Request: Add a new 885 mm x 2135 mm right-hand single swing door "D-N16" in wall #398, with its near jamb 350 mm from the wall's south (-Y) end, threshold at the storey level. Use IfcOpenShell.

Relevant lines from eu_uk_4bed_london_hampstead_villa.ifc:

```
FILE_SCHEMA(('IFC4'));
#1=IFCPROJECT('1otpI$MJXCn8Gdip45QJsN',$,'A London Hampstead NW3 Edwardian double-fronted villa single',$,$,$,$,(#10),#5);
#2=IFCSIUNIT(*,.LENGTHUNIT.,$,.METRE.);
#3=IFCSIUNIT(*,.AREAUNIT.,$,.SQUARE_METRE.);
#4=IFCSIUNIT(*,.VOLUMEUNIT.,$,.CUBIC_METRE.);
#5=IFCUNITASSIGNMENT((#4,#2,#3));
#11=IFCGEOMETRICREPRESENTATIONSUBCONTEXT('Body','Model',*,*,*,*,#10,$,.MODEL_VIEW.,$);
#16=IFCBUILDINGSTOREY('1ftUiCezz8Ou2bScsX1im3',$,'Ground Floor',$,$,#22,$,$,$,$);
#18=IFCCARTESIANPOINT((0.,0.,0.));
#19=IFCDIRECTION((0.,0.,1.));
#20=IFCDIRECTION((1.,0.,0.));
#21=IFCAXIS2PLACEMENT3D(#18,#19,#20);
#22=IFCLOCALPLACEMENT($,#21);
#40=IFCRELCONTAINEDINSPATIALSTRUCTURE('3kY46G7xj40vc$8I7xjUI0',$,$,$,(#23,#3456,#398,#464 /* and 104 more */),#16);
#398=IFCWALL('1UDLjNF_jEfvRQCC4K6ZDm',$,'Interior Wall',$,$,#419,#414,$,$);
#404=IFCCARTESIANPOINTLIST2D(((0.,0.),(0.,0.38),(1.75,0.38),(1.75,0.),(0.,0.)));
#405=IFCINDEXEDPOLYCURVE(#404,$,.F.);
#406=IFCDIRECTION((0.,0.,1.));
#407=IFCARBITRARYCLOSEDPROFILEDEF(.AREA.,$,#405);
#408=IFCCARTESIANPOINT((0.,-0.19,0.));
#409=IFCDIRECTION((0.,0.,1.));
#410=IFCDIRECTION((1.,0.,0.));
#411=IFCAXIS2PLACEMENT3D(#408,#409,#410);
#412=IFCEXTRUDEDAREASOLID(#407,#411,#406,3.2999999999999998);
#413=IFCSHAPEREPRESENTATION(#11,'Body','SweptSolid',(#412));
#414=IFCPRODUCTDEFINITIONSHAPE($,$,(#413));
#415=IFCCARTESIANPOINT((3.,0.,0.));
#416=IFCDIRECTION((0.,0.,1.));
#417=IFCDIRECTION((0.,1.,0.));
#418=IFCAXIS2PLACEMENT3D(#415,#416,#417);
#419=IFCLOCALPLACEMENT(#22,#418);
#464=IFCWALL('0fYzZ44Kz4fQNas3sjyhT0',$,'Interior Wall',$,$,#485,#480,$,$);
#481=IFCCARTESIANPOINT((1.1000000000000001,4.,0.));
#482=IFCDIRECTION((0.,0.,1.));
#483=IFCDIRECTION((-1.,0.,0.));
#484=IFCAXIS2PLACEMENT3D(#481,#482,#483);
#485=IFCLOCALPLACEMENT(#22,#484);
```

```python
import numpy as np
import ifcopenshell
import ifcopenshell.api.feature
import ifcopenshell.api.geometry
import ifcopenshell.api.root
import ifcopenshell.api.spatial
import ifcopenshell.geom
import ifcopenshell.util.element
import ifcopenshell.util.placement
import ifcopenshell.util.representation
import ifcopenshell.util.shape
import ifcopenshell.util.unit

model = ifcopenshell.open("eu_uk_4bed_london_hampstead_villa.ifc")
unit_scale = ifcopenshell.util.unit.calculate_unit_scale(model)
settings = ifcopenshell.geom.settings()


def volume(element):
    """Net volume in cubic metres, openings subtracted."""
    shape = ifcopenshell.geom.create_shape(settings, element)
    return ifcopenshell.util.shape.get_volume(shape.geometry)


wall = model.by_guid("1UDLjNF_jEfvRQCC4K6ZDm")
storey = ifcopenshell.util.element.get_container(wall, ifc_class="IfcBuildingStorey")
context = ifcopenshell.util.representation.get_context(model, "Model", "Body", "MODEL_VIEW")
before = volume(wall)

width, height, from_end, sill = 0.885, 2.135, 0.35, 0.0  # metres

# The wall runs along its own X axis, and the end named is its -X end.
wall_shape = ifcopenshell.geom.create_shape(settings, wall)
x, y, z = ifcopenshell.util.shape.get_vertices(wall_shape.geometry).T
start = x.min() + from_end
face, thickness = float(y.min()), float(y.max() - y.min())
wall_matrix = ifcopenshell.util.placement.get_local_placement(wall.ObjectPlacement)
level = ifcopenshell.util.placement.get_local_placement(storey.ObjectPlacement)[2, 3]


def in_wall(x, y):
    """Placement at x, y metres in the wall's axes, at sill height."""
    matrix = wall_matrix.copy()
    matrix[:, 3] = wall_matrix @ np.array([x / unit_scale, y / unit_scale, 0.0, 1.0])
    matrix[2, 3] = level + sill / unit_scale
    return matrix


# Opening: a box that overshoots both wall faces by 50 mm.
opening = ifcopenshell.api.root.create_entity(model, ifc_class="IfcOpeningElement", predefined_type="OPENING")
box = ifcopenshell.api.geometry.add_wall_representation(
    model, context=context, length=width, height=height, thickness=thickness + 0.1
)
ifcopenshell.api.geometry.assign_representation(model, product=opening, representation=box)
ifcopenshell.api.geometry.edit_object_placement(model, product=opening, matrix=in_wall(start, face - 0.05), is_si=False)
ifcopenshell.api.feature.add_feature(model, feature=opening, element=wall)

door = ifcopenshell.api.root.create_entity(model, ifc_class="IfcDoor", name="D-N16", predefined_type="DOOR")
door.OverallWidth, door.OverallHeight = width / unit_scale, height / unit_scale
door.OperationType = "SINGLE_SWING_RIGHT"
body = ifcopenshell.api.geometry.add_door_representation(
    model,
    context=context,
    overall_width=door.OverallWidth,
    overall_height=door.OverallHeight,
    operation_type="SINGLE_SWING_RIGHT",
    lining_properties={"LiningDepth": thickness / unit_scale, "ThresholdDepth": thickness / unit_scale},
)
ifcopenshell.api.geometry.assign_representation(model, product=door, representation=body)
ifcopenshell.api.spatial.assign_container(model, products=[door], relating_structure=storey)
ifcopenshell.api.feature.add_filling(model, opening=opening, element=door)

# The lining spans the wall, so the door starts at the wall face.
ifcopenshell.api.geometry.edit_object_placement(model, product=door, matrix=in_wall(start, face), is_si=False)

after = volume(wall)

print(f"wall volume {before:.3f} -> {after:.3f} m3")

model.write("eu_uk_4bed_london_hampstead_villa_rev.ifc")
```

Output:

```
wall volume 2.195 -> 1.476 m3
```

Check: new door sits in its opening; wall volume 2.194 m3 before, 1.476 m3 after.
